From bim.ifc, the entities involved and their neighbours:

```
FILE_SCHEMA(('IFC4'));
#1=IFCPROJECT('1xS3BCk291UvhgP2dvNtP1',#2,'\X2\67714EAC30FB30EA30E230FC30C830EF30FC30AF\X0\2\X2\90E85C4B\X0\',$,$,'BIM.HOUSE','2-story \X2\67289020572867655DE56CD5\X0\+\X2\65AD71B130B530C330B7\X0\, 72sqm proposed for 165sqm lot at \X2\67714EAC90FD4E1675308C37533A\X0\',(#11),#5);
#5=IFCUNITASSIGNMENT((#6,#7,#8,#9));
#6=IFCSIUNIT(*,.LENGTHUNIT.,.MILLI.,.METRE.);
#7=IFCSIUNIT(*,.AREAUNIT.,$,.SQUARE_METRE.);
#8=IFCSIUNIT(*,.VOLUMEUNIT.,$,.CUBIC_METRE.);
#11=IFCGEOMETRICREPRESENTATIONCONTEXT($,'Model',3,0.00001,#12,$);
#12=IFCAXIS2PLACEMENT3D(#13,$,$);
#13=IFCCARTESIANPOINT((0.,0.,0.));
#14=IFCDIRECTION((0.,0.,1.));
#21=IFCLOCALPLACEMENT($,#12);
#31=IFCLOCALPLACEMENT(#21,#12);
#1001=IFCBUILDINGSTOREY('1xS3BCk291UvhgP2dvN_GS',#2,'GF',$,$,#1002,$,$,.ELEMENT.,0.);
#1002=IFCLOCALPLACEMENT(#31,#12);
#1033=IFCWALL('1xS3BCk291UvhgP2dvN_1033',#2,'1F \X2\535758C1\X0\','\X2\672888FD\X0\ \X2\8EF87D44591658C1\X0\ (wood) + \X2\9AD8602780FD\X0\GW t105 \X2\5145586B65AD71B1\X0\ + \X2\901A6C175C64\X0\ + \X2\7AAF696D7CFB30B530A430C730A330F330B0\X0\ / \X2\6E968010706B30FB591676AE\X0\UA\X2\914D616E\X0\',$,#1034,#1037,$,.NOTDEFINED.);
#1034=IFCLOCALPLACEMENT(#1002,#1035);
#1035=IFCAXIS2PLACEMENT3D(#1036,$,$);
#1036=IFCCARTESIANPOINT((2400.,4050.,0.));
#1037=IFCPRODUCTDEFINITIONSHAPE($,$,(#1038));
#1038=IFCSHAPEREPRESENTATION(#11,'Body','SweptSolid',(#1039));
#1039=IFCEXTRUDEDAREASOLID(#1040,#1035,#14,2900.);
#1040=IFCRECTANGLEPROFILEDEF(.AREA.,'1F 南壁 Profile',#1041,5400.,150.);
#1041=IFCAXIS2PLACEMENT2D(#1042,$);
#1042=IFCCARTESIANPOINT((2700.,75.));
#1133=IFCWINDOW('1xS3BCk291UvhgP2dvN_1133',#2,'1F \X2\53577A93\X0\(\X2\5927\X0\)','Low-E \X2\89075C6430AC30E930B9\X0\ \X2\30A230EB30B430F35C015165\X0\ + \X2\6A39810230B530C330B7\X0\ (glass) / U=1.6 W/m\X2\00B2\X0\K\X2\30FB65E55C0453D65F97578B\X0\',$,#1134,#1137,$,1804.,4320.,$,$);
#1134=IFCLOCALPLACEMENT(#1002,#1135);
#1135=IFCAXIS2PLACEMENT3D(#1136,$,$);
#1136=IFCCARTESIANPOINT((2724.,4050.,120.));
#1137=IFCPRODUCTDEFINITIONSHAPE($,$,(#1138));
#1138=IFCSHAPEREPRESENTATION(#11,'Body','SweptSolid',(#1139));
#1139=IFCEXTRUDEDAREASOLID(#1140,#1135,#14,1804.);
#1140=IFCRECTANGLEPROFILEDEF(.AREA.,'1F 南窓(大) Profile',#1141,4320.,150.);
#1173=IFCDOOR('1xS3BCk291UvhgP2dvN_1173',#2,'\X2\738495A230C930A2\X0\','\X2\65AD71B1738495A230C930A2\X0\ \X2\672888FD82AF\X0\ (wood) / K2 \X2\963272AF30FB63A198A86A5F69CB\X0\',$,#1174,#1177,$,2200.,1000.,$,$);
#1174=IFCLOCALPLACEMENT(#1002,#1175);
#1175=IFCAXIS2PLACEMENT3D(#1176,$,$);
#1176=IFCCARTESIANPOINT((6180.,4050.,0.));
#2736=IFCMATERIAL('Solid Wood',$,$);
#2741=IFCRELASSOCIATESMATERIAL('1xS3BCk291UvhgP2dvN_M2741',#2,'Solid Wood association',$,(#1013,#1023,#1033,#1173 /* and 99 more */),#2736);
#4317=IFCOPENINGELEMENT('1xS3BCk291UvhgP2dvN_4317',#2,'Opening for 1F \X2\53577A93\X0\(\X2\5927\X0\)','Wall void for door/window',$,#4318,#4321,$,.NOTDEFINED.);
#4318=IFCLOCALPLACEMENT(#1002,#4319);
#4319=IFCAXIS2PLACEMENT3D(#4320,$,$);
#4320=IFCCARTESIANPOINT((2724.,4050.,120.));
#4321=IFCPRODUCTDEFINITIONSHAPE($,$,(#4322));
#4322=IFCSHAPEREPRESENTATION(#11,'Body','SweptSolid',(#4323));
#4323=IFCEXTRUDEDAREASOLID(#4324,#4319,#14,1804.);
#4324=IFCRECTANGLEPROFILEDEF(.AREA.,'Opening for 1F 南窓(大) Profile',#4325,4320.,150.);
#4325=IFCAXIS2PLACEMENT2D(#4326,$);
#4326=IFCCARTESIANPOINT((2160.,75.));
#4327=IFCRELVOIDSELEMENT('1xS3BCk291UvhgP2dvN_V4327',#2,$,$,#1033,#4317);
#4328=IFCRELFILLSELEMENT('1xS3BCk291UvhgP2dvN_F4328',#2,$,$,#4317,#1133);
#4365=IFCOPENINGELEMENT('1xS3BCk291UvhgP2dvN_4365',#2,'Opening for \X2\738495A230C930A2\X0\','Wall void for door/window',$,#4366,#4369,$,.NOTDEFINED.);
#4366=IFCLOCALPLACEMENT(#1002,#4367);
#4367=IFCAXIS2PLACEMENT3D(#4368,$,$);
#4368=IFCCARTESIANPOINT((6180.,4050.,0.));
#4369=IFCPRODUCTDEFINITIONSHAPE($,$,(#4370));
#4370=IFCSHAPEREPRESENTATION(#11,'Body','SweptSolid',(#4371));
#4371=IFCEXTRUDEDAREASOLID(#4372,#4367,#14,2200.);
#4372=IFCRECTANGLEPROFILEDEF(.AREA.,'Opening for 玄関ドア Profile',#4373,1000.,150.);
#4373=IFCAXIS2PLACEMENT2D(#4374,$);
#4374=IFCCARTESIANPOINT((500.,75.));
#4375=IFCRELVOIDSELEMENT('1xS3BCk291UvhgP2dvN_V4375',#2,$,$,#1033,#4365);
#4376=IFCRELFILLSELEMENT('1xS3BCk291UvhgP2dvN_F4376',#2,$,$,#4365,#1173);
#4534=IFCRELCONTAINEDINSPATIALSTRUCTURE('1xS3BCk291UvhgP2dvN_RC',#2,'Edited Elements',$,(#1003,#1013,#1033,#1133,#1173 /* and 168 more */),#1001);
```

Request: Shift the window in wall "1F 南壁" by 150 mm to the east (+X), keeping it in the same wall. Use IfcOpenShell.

```python
import ifcopenshell
import ifcopenshell.api.geometry
import ifcopenshell.util.placement
import ifcopenshell.util.unit

model = ifcopenshell.open("bim.ifc")
unit_scale = ifcopenshell.util.unit.calculate_unit_scale(model)

window = model.by_id(1133)
opening = window.FillsVoids[0].RelatingOpeningElement
wall = opening.VoidsElements[0].RelatingBuildingElement

wall_matrix = ifcopenshell.util.placement.get_local_placement(wall.ObjectPlacement)
shift = wall_matrix[:3, 0] * 0.15 / unit_scale
before = ifcopenshell.util.placement.get_local_placement(window.ObjectPlacement)[:3, 3].copy()

# The window is not placed relative to its opening, so move both.
for product in (opening, window):
    matrix = ifcopenshell.util.placement.get_local_placement(product.ObjectPlacement)
    matrix[:3, 3] += shift
    ifcopenshell.api.geometry.edit_object_placement(model, product=product, matrix=matrix, is_si=False)

after = ifcopenshell.util.placement.get_local_placement(window.ObjectPlacement)[:3, 3]
print("window moved by", (after - before).round(3) + 0.0)

model.write("bim_rev.ifc")
```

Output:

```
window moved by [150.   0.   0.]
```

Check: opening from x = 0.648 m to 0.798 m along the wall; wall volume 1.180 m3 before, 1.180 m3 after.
